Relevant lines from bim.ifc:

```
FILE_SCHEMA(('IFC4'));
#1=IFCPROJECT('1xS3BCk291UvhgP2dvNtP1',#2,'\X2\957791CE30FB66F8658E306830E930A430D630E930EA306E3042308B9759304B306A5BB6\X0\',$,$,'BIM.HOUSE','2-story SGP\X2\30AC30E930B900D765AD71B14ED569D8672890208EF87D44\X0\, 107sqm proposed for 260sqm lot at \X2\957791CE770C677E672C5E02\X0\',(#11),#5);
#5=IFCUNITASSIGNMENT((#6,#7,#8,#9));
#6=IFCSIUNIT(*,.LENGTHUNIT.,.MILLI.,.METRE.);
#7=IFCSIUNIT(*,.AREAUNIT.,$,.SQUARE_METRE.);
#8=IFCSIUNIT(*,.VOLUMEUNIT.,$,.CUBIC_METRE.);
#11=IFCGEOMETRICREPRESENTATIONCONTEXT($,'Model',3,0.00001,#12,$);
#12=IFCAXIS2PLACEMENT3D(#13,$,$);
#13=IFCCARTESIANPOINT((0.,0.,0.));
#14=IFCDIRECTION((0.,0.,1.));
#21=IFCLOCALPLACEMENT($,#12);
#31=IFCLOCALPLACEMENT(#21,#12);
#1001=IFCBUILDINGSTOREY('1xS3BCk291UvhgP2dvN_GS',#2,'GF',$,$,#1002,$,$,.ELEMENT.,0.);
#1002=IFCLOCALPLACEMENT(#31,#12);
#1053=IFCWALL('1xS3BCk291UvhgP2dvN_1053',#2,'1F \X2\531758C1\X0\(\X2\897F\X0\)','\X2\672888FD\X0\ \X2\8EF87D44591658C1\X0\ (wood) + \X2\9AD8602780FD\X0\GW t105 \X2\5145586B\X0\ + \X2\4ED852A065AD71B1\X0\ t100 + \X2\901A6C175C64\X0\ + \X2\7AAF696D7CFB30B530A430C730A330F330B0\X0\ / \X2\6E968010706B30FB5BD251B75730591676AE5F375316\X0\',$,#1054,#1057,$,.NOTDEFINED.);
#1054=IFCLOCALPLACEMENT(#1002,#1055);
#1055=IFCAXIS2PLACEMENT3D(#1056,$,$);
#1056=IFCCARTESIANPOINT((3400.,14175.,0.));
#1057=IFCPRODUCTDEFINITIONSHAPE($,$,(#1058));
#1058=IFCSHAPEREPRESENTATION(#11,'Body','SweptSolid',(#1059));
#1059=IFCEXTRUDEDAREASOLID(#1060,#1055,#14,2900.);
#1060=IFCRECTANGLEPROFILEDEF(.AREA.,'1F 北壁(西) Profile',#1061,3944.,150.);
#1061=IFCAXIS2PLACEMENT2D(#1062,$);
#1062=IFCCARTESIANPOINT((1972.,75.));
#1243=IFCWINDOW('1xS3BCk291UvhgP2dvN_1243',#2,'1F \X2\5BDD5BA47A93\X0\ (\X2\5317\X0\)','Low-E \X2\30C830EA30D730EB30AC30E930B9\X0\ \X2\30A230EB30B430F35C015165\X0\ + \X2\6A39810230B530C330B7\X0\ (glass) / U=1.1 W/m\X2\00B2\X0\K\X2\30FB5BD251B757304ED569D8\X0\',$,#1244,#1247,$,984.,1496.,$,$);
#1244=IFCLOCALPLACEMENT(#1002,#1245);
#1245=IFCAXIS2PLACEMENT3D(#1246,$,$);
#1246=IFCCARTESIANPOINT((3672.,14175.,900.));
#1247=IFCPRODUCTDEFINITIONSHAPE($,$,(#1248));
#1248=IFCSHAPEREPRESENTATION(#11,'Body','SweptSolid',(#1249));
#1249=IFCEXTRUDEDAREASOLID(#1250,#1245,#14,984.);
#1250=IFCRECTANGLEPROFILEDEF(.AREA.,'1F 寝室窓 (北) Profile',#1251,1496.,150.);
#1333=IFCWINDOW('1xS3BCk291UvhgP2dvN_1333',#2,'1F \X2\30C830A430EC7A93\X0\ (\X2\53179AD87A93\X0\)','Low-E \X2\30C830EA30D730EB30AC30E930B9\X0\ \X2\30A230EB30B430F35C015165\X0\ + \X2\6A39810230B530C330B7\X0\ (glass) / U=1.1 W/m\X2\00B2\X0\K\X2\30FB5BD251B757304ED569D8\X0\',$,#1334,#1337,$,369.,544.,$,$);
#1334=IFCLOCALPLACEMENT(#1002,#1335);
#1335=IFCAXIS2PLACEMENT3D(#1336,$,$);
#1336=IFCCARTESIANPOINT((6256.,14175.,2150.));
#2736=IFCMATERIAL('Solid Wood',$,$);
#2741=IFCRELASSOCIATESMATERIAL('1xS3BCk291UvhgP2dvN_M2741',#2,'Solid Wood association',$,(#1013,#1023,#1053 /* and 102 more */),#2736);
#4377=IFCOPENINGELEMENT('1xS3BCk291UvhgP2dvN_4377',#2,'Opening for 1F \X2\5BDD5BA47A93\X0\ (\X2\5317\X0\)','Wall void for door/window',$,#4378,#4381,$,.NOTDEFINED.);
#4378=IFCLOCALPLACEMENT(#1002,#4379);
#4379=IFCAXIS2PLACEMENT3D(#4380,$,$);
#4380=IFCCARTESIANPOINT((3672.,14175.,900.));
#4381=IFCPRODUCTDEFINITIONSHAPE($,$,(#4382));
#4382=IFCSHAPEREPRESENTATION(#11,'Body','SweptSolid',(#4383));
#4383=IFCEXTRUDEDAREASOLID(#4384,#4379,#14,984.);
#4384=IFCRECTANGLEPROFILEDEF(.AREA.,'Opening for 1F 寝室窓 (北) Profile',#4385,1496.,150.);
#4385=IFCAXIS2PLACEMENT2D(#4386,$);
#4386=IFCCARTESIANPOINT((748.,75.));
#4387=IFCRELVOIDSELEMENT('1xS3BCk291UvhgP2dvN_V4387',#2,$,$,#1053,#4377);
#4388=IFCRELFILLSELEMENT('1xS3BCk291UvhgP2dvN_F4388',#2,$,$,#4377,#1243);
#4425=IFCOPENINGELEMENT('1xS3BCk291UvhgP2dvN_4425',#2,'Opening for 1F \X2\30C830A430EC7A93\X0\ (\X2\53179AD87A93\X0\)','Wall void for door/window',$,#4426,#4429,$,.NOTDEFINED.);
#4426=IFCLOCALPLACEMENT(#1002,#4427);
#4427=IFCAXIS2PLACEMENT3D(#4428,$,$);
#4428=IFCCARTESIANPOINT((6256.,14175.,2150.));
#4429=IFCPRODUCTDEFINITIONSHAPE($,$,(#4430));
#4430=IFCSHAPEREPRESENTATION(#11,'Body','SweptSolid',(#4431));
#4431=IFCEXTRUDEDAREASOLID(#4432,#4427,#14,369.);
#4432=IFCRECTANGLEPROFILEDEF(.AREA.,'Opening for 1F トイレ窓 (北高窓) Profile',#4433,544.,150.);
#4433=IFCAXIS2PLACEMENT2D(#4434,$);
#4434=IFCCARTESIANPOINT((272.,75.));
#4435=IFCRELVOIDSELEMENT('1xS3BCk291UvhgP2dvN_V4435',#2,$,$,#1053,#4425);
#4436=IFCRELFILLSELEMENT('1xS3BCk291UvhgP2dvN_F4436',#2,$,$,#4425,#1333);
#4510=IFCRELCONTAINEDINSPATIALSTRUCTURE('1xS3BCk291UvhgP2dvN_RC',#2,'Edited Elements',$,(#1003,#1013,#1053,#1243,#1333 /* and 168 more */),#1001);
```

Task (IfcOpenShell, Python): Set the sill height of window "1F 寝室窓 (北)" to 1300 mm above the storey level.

```python
import numpy as np
import ifcopenshell
import ifcopenshell.api.geometry
import ifcopenshell.geom
import ifcopenshell.util.element
import ifcopenshell.util.placement
import ifcopenshell.util.shape
import ifcopenshell.util.unit

model = ifcopenshell.open("bim.ifc")
unit_scale = ifcopenshell.util.unit.calculate_unit_scale(model)

window = model.by_id(1243)
opening = window.FillsVoids[0].RelatingOpeningElement
storey = ifcopenshell.util.element.get_container(window, ifc_class="IfcBuildingStorey")
level = ifcopenshell.util.placement.get_local_placement(storey.ObjectPlacement)[2, 3]

# The opening's origin need not be at the sill, so measure its lowest point.
shape = ifcopenshell.geom.create_shape(ifcopenshell.geom.settings(), opening)
bottom = ifcopenshell.util.shape.get_shape_bottom_elevation(shape, shape.geometry) / unit_scale
dz = level + 1300.0 - bottom

shift = np.array([0.0, 0.0, dz])
# The window is not placed relative to its opening, so move both.
for product in (opening, window):
    matrix = ifcopenshell.util.placement.get_local_placement(product.ObjectPlacement)
    matrix[:3, 3] += shift
    ifcopenshell.api.geometry.edit_object_placement(model, product=product, matrix=matrix, is_si=False)

print(f"moved by {dz * unit_scale:+.3f} m")

model.write("bim_rev.ifc")
```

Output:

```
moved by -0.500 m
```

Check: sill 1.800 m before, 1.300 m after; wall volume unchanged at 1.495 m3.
